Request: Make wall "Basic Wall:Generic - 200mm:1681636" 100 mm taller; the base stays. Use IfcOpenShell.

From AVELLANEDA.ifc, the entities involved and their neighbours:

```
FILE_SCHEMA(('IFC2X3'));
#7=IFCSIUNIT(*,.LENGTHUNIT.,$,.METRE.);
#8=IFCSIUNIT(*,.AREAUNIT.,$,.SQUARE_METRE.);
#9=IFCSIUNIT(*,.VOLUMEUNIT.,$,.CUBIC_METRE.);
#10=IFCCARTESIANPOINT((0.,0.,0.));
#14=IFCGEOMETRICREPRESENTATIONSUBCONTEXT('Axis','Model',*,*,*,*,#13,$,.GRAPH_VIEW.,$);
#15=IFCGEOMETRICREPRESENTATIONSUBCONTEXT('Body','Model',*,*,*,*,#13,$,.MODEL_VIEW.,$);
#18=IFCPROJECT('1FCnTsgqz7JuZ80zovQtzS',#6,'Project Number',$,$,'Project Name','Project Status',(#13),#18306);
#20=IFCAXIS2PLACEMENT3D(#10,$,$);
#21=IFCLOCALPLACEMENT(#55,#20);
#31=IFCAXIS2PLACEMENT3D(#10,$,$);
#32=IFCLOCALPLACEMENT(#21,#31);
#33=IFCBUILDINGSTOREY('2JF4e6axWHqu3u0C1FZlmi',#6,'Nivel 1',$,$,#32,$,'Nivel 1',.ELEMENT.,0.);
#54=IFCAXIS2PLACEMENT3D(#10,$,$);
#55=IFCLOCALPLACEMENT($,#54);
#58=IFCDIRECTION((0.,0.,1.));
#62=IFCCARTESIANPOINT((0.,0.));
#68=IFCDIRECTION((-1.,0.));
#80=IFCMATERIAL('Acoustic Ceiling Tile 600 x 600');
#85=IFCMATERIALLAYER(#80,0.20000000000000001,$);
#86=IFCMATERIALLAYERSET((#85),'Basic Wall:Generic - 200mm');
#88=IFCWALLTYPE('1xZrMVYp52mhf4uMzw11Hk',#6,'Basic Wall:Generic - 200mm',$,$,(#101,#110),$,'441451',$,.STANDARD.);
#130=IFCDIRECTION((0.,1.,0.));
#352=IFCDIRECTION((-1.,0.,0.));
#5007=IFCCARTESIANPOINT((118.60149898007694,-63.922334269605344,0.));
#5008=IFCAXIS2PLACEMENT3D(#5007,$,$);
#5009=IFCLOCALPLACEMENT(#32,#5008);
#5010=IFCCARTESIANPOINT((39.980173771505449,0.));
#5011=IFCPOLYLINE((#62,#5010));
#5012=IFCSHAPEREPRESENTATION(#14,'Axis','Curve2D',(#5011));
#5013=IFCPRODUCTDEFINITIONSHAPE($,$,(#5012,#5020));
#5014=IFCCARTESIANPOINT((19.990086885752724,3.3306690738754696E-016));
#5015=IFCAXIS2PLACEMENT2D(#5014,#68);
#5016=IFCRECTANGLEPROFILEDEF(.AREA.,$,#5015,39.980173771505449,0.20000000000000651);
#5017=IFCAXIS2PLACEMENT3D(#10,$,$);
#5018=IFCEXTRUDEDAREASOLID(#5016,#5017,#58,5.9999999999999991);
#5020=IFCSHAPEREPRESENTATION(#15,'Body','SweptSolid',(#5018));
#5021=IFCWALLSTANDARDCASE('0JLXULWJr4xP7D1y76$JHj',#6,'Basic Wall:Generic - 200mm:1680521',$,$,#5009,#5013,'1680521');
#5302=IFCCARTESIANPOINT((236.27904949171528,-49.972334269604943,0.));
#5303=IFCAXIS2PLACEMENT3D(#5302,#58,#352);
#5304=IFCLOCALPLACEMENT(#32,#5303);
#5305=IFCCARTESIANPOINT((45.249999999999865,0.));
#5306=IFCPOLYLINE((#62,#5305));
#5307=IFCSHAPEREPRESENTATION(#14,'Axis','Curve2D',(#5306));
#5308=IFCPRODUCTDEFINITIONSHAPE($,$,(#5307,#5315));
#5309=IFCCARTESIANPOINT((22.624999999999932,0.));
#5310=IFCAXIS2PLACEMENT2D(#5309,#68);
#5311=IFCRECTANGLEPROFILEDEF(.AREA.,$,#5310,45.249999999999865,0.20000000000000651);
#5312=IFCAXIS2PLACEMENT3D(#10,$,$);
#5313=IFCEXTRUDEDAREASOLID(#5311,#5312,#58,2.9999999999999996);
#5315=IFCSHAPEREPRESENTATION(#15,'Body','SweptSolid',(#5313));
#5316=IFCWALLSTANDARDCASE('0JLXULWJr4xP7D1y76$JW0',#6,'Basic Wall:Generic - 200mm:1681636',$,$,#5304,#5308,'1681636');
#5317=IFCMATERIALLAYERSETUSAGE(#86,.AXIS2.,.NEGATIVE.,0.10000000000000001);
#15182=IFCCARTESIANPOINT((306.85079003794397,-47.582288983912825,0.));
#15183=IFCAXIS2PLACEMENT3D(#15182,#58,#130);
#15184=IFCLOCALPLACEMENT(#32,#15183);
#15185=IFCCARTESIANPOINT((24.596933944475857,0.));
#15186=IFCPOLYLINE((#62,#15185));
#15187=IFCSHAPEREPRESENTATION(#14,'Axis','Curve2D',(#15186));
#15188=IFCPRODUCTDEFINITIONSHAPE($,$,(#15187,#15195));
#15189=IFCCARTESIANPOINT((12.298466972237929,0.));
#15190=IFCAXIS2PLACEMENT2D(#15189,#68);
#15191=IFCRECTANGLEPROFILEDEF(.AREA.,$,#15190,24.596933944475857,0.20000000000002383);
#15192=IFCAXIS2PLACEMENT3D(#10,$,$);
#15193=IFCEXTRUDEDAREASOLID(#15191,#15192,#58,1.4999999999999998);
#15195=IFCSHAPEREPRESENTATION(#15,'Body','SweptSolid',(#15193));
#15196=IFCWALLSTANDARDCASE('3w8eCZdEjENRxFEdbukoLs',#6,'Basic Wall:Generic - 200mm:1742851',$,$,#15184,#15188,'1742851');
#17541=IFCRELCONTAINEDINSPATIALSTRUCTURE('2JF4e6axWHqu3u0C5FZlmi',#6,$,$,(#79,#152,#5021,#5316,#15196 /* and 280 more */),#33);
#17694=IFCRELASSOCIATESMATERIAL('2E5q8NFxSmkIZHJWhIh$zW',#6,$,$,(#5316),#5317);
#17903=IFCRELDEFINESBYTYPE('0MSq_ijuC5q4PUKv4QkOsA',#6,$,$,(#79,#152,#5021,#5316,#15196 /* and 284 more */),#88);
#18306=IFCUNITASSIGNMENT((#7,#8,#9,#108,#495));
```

```python
import ifcopenshell
import ifcopenshell.geom
import ifcopenshell.util.representation
import ifcopenshell.util.shape

model = ifcopenshell.open("AVELLANEDA.ifc")
settings = ifcopenshell.geom.settings()


def volume(element):
    """Net volume in cubic metres, openings subtracted."""
    shape = ifcopenshell.geom.create_shape(settings, element)
    return ifcopenshell.util.shape.get_volume(shape.geometry)


wall = model.by_guid("0JLXULWJr4xP7D1y76$JW0")
before = volume(wall)

body = ifcopenshell.util.representation.get_representation(wall, "Model", "Body")
solid = body.Items[0]
old_height = solid.Depth
solid.Depth += 0.1
after = volume(wall)

print(f"height {old_height:g} -> {solid.Depth:g}, volume {before:.3f} -> {after:.3f} m3")

model.write("AVELLANEDA_edited.ifc")
```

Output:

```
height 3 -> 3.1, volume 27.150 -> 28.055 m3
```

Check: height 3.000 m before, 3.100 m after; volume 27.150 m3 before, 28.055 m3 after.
